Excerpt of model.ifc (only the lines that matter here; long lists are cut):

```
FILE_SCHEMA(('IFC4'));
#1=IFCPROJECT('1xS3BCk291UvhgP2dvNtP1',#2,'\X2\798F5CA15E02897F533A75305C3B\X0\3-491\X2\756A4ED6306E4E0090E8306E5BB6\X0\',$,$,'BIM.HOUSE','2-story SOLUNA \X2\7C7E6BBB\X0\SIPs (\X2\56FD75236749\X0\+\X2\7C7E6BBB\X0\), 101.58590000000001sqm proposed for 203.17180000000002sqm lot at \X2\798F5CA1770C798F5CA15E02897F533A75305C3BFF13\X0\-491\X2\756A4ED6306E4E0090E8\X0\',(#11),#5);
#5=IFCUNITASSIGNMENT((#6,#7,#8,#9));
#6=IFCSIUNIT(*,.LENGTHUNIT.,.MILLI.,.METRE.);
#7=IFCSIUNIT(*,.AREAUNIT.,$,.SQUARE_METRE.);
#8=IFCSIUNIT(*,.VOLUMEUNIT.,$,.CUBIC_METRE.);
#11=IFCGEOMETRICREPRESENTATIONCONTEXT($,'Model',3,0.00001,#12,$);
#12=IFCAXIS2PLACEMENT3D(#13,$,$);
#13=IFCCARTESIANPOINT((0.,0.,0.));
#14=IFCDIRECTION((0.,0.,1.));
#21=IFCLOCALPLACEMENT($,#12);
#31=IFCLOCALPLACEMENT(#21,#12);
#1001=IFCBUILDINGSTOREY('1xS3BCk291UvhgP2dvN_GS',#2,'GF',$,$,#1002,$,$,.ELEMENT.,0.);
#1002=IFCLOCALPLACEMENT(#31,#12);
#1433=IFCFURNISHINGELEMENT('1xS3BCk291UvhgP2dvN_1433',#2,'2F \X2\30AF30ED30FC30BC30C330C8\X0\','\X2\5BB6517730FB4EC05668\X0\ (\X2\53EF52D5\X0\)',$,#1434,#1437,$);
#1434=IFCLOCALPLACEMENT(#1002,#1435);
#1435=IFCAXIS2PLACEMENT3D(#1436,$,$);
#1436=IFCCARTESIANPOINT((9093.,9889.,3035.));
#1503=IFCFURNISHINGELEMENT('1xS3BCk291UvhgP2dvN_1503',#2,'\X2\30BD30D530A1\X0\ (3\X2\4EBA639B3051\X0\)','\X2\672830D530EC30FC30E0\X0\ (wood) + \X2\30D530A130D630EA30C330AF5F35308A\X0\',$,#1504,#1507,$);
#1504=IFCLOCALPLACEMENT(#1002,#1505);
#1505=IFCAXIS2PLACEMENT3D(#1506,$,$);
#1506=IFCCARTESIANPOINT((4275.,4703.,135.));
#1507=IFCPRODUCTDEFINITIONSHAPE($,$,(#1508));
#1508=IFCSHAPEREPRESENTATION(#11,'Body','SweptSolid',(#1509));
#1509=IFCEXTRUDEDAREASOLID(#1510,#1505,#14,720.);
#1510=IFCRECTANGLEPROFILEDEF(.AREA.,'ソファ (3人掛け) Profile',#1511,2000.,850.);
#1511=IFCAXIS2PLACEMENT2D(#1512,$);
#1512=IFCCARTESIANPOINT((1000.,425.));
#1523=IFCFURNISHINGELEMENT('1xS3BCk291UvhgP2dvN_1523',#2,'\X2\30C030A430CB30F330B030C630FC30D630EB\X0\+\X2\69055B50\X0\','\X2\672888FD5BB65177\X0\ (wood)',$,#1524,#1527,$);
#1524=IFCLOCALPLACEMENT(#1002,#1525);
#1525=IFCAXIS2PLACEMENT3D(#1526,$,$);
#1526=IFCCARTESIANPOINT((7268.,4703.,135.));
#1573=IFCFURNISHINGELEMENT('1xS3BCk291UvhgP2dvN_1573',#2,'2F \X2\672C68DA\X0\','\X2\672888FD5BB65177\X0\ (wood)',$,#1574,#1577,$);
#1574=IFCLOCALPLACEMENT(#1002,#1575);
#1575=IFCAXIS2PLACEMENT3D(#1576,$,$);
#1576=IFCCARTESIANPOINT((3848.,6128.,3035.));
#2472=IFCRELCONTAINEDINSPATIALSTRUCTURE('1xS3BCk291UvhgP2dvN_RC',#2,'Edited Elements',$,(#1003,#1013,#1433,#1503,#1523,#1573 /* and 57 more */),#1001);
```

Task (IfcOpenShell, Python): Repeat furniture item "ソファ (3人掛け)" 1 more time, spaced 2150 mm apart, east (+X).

```python
import numpy as np
import ifcopenshell
import ifcopenshell.api.geometry
import ifcopenshell.api.root
import ifcopenshell.util.element
import ifcopenshell.util.placement
import ifcopenshell.util.unit

model = ifcopenshell.open("model.ifc")
unit_scale = ifcopenshell.util.unit.calculate_unit_scale(model)


def reuse_history(source, copy):
    """copy_class also copies each property set's owner history, people and application; keep the originals."""
    for rel in copy.IsDefinedBy:
        if rel.is_a("IfcRelDefinesByProperties") and (history := rel.RelatingPropertyDefinition.OwnerHistory):
            rel.RelatingPropertyDefinition.OwnerHistory = source.OwnerHistory
            ifcopenshell.util.element.remove_deep2(model, history)


source = model.by_guid("1xS3BCk291UvhgP2dvN_1503")
base = ifcopenshell.util.placement.get_local_placement(source.ObjectPlacement)
step = np.array([1.0, 0.0, 0.0]) * 2.15 / unit_scale

for i in range(1, 2):
    copy = ifcopenshell.api.root.copy_class(model, product=source)
    copy.Representation = ifcopenshell.util.element.copy_deep(
        model, source.Representation, exclude=["IfcGeometricRepresentationContext", "IfcRepresentationMap"]
    )
    reuse_history(source, copy)
    matrix = base.copy()
    matrix[:3, 3] += i * step
    print("added at", matrix[:3, 3].round(3) + 0.0)
    ifcopenshell.api.geometry.edit_object_placement(model, product=copy, matrix=matrix, is_si=False)

model.write("model_updated.ifc")
```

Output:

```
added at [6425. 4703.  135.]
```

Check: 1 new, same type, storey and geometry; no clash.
